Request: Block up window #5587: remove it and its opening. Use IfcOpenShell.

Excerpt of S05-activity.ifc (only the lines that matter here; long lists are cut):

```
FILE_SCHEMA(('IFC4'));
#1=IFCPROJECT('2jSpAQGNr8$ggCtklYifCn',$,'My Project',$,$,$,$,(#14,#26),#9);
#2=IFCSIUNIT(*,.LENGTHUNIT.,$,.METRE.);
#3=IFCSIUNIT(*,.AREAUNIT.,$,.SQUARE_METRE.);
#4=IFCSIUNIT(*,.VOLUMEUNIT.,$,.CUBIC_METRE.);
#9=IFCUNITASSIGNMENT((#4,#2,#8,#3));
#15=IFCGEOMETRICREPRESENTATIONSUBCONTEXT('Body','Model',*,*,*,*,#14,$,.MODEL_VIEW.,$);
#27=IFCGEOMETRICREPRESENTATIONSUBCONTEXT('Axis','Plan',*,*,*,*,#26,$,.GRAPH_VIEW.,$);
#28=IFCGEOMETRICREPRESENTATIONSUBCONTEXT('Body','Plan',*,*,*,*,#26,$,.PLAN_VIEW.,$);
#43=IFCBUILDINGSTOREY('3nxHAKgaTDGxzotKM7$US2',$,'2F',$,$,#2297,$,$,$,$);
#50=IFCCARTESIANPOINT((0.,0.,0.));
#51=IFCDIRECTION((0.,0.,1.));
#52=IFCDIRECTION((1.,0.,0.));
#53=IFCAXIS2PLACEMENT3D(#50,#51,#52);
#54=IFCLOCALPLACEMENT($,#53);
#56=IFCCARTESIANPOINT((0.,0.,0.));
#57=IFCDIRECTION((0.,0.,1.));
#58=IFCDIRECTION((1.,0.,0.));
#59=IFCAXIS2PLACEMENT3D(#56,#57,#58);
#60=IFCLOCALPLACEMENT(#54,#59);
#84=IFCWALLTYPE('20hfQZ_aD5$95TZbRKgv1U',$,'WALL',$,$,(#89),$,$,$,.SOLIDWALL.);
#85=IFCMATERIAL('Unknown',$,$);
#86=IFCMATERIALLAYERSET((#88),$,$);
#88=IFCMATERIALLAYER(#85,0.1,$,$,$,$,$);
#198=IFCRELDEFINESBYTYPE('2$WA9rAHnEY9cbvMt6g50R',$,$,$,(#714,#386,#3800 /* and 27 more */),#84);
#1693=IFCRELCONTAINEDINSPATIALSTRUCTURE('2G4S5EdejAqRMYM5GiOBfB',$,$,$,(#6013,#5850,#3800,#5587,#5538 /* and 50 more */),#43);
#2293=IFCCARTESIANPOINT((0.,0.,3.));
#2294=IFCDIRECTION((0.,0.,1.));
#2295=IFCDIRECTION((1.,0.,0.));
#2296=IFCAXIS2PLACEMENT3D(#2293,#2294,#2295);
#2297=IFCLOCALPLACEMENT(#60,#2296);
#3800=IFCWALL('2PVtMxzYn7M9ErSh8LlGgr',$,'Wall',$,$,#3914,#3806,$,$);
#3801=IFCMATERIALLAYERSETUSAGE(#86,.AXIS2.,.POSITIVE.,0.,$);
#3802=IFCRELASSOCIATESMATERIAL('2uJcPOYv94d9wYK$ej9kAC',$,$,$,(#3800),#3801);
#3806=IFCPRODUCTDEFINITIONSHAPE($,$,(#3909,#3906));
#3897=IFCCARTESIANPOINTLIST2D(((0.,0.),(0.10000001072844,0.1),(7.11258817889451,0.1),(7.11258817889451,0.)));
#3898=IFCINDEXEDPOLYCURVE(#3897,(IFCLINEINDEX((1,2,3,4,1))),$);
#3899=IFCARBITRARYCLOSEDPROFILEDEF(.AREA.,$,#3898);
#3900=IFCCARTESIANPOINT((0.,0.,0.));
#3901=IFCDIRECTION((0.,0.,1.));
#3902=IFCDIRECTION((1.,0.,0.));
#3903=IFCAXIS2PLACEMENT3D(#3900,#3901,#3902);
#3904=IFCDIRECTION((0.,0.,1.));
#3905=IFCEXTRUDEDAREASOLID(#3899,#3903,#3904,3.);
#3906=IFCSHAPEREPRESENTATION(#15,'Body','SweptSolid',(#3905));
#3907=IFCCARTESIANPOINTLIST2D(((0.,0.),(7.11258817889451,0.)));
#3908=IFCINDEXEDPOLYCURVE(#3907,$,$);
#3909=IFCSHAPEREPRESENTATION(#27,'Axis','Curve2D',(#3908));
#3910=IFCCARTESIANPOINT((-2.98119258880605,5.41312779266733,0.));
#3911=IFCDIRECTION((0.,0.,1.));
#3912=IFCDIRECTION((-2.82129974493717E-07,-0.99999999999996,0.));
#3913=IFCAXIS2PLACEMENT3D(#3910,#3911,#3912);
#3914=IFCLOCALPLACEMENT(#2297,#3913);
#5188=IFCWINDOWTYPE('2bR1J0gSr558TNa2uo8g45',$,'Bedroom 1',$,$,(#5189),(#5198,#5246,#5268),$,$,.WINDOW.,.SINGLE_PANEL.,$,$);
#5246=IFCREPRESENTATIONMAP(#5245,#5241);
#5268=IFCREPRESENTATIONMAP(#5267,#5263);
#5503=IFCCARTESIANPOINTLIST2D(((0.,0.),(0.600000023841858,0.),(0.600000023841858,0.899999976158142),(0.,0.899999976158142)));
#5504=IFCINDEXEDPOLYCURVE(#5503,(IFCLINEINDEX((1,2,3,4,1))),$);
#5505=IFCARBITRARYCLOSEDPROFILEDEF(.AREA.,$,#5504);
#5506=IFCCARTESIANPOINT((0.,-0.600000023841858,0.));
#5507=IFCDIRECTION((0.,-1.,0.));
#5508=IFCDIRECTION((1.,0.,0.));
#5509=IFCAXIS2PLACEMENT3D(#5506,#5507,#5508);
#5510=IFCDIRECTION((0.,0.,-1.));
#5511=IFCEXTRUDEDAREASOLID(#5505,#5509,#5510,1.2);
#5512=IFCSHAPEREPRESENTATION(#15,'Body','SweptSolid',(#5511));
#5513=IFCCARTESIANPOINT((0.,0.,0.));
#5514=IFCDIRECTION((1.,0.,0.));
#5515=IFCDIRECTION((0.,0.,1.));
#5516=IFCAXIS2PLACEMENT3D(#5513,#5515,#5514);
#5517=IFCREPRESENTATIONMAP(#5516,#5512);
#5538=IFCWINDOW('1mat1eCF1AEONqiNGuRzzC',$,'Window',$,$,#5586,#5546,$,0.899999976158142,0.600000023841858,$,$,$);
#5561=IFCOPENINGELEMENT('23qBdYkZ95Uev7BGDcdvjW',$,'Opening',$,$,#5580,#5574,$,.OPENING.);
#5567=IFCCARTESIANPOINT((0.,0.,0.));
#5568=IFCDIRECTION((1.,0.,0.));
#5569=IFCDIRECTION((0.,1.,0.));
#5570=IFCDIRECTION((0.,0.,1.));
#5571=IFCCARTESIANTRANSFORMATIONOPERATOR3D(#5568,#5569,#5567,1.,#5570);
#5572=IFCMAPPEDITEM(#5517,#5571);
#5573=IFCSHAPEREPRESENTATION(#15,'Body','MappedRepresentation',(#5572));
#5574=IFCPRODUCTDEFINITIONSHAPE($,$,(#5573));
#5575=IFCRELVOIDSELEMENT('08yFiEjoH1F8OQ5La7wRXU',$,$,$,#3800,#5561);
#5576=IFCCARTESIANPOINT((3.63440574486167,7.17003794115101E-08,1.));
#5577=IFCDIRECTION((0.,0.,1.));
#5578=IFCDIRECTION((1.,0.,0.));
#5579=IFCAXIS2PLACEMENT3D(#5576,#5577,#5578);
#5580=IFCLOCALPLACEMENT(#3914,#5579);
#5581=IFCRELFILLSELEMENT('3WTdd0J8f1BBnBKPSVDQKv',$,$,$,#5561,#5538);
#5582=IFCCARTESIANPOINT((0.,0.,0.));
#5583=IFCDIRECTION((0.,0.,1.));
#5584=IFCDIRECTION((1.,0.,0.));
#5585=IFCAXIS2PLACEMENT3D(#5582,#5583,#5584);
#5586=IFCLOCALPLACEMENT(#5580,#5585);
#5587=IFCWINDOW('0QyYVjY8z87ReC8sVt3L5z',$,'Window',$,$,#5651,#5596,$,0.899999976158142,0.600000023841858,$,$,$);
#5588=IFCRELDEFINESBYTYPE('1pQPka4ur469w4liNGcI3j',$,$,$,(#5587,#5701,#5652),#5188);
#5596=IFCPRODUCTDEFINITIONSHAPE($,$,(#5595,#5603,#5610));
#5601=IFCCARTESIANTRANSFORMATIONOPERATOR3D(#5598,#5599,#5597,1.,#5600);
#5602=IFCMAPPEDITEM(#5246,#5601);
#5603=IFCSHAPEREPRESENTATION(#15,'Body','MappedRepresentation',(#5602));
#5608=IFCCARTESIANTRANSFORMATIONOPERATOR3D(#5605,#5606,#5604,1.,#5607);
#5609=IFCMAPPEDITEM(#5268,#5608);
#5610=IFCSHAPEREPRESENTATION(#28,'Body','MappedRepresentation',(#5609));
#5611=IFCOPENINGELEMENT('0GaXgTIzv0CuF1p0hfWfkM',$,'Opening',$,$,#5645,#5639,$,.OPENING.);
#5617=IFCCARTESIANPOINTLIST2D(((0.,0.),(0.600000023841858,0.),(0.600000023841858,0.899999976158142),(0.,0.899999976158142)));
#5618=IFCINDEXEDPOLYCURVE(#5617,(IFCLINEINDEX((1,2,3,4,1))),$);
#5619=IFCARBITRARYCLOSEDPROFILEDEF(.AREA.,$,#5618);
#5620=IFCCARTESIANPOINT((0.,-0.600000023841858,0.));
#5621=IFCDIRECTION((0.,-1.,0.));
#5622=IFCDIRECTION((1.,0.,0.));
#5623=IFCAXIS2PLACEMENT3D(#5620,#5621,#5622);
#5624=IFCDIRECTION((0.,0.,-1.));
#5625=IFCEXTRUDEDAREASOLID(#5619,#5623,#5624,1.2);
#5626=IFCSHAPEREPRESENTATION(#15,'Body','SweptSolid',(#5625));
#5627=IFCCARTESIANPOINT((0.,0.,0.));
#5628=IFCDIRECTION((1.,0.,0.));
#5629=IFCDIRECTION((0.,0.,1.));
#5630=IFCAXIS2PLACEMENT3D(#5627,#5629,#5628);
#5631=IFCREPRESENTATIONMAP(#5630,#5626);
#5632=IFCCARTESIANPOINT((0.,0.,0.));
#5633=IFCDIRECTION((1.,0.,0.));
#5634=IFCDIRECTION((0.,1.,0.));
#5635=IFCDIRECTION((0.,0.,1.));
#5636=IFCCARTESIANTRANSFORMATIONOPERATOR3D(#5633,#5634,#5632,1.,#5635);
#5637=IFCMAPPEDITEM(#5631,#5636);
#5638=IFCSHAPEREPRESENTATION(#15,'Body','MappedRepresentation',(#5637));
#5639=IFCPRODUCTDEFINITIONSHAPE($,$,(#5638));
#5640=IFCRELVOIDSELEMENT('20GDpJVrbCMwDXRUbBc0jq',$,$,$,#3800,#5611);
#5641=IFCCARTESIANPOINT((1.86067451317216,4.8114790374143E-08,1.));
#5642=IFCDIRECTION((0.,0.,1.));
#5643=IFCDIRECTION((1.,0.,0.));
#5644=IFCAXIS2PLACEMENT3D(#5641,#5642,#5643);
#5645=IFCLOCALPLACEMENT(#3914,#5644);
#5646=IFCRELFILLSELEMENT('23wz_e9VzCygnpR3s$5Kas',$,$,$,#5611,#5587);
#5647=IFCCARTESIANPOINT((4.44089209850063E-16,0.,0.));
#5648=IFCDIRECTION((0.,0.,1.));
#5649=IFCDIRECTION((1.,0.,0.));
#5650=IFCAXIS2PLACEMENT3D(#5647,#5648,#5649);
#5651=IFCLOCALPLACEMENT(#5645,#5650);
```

```python
import ifcopenshell
import ifcopenshell.api.feature
import ifcopenshell.api.root
import ifcopenshell.geom
import ifcopenshell.util.shape

model = ifcopenshell.open("S05-activity.ifc")
settings = ifcopenshell.geom.settings()


def volume(element):
    """Net volume in cubic metres, openings subtracted."""
    shape = ifcopenshell.geom.create_shape(settings, element)
    return ifcopenshell.util.shape.get_volume(shape.geometry)


window = model.by_id(5587)
opening = window.FillsVoids[0].RelatingOpeningElement
wall = opening.VoidsElements[0].RelatingBuildingElement
before = volume(wall)

ifcopenshell.api.root.remove_product(model, product=window)
ifcopenshell.api.feature.remove_feature(model, feature=opening)

after = volume(wall)

print(f"wall volume {before:.3f} -> {after:.3f} m3")

model.write("S05-activity_v2.ifc")
```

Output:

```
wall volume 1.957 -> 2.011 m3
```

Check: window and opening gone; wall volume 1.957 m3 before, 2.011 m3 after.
